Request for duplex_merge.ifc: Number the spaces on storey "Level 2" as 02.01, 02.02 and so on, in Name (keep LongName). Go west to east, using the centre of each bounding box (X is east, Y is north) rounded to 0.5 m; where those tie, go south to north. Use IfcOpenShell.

First a look at what the model holds.

```python
import ifcopenshell
import ifcopenshell.util.element
import ifcopenshell.util.placement

model = ifcopenshell.open("duplex_merge.ifc")
print(model.schema)
storey = next(s for s in model.by_type("IfcBuildingStorey") if s.Name == "Level 2")
spaces = [e for e in ifcopenshell.util.element.get_decomposition(storey) if e.is_a("IfcSpace")]
for e in sorted(spaces, key=lambda e: e.id()):
    origin = ifcopenshell.util.placement.get_local_placement(e.ObjectPlacement)[:3, 3]
    print(e.id(), e.Name, e.LongName, origin.round(2) + 0.0, sep=" | ")
```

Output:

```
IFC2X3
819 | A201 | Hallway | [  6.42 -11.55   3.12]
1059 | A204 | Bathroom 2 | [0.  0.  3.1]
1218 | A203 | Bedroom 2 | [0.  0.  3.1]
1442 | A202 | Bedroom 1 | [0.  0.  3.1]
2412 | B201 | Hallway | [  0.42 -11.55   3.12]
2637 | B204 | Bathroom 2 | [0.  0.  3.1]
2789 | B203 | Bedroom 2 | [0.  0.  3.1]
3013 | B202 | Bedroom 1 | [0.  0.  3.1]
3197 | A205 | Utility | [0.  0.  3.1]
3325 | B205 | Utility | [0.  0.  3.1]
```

```python
import ifcopenshell
import ifcopenshell.geom
import ifcopenshell.util.element
import ifcopenshell.util.shape

model = ifcopenshell.open("duplex_merge.ifc")
settings = ifcopenshell.geom.settings()
settings.set("use-world-coords", True)


def centre(element):
    shape = ifcopenshell.geom.create_shape(settings, element)
    return ifcopenshell.util.shape.get_bbox_centroid(shape.geometry)


storey = next(s for s in model.by_type("IfcBuildingStorey") if s.Name == "Level 2")
spaces = [e for e in ifcopenshell.util.element.get_decomposition(storey) if e.is_a("IfcSpace")]

# Insertion points can sit at a corner or the storey origin, so sort by the geometry (in metres).
centres = {e: centre(e) for e in spaces}
spaces.sort(key=lambda e: (round(centres[e][0] / 0.5), centres[e][1]))

for i, e in enumerate(spaces, start=1):
    number = f"02.{i:02d}"
    e.Name = number
    print(e.id(), number)

model.write("duplex_merge-out.ifc")
```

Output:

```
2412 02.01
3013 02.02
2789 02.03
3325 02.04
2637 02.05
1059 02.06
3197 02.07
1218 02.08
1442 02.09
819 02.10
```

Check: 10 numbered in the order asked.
